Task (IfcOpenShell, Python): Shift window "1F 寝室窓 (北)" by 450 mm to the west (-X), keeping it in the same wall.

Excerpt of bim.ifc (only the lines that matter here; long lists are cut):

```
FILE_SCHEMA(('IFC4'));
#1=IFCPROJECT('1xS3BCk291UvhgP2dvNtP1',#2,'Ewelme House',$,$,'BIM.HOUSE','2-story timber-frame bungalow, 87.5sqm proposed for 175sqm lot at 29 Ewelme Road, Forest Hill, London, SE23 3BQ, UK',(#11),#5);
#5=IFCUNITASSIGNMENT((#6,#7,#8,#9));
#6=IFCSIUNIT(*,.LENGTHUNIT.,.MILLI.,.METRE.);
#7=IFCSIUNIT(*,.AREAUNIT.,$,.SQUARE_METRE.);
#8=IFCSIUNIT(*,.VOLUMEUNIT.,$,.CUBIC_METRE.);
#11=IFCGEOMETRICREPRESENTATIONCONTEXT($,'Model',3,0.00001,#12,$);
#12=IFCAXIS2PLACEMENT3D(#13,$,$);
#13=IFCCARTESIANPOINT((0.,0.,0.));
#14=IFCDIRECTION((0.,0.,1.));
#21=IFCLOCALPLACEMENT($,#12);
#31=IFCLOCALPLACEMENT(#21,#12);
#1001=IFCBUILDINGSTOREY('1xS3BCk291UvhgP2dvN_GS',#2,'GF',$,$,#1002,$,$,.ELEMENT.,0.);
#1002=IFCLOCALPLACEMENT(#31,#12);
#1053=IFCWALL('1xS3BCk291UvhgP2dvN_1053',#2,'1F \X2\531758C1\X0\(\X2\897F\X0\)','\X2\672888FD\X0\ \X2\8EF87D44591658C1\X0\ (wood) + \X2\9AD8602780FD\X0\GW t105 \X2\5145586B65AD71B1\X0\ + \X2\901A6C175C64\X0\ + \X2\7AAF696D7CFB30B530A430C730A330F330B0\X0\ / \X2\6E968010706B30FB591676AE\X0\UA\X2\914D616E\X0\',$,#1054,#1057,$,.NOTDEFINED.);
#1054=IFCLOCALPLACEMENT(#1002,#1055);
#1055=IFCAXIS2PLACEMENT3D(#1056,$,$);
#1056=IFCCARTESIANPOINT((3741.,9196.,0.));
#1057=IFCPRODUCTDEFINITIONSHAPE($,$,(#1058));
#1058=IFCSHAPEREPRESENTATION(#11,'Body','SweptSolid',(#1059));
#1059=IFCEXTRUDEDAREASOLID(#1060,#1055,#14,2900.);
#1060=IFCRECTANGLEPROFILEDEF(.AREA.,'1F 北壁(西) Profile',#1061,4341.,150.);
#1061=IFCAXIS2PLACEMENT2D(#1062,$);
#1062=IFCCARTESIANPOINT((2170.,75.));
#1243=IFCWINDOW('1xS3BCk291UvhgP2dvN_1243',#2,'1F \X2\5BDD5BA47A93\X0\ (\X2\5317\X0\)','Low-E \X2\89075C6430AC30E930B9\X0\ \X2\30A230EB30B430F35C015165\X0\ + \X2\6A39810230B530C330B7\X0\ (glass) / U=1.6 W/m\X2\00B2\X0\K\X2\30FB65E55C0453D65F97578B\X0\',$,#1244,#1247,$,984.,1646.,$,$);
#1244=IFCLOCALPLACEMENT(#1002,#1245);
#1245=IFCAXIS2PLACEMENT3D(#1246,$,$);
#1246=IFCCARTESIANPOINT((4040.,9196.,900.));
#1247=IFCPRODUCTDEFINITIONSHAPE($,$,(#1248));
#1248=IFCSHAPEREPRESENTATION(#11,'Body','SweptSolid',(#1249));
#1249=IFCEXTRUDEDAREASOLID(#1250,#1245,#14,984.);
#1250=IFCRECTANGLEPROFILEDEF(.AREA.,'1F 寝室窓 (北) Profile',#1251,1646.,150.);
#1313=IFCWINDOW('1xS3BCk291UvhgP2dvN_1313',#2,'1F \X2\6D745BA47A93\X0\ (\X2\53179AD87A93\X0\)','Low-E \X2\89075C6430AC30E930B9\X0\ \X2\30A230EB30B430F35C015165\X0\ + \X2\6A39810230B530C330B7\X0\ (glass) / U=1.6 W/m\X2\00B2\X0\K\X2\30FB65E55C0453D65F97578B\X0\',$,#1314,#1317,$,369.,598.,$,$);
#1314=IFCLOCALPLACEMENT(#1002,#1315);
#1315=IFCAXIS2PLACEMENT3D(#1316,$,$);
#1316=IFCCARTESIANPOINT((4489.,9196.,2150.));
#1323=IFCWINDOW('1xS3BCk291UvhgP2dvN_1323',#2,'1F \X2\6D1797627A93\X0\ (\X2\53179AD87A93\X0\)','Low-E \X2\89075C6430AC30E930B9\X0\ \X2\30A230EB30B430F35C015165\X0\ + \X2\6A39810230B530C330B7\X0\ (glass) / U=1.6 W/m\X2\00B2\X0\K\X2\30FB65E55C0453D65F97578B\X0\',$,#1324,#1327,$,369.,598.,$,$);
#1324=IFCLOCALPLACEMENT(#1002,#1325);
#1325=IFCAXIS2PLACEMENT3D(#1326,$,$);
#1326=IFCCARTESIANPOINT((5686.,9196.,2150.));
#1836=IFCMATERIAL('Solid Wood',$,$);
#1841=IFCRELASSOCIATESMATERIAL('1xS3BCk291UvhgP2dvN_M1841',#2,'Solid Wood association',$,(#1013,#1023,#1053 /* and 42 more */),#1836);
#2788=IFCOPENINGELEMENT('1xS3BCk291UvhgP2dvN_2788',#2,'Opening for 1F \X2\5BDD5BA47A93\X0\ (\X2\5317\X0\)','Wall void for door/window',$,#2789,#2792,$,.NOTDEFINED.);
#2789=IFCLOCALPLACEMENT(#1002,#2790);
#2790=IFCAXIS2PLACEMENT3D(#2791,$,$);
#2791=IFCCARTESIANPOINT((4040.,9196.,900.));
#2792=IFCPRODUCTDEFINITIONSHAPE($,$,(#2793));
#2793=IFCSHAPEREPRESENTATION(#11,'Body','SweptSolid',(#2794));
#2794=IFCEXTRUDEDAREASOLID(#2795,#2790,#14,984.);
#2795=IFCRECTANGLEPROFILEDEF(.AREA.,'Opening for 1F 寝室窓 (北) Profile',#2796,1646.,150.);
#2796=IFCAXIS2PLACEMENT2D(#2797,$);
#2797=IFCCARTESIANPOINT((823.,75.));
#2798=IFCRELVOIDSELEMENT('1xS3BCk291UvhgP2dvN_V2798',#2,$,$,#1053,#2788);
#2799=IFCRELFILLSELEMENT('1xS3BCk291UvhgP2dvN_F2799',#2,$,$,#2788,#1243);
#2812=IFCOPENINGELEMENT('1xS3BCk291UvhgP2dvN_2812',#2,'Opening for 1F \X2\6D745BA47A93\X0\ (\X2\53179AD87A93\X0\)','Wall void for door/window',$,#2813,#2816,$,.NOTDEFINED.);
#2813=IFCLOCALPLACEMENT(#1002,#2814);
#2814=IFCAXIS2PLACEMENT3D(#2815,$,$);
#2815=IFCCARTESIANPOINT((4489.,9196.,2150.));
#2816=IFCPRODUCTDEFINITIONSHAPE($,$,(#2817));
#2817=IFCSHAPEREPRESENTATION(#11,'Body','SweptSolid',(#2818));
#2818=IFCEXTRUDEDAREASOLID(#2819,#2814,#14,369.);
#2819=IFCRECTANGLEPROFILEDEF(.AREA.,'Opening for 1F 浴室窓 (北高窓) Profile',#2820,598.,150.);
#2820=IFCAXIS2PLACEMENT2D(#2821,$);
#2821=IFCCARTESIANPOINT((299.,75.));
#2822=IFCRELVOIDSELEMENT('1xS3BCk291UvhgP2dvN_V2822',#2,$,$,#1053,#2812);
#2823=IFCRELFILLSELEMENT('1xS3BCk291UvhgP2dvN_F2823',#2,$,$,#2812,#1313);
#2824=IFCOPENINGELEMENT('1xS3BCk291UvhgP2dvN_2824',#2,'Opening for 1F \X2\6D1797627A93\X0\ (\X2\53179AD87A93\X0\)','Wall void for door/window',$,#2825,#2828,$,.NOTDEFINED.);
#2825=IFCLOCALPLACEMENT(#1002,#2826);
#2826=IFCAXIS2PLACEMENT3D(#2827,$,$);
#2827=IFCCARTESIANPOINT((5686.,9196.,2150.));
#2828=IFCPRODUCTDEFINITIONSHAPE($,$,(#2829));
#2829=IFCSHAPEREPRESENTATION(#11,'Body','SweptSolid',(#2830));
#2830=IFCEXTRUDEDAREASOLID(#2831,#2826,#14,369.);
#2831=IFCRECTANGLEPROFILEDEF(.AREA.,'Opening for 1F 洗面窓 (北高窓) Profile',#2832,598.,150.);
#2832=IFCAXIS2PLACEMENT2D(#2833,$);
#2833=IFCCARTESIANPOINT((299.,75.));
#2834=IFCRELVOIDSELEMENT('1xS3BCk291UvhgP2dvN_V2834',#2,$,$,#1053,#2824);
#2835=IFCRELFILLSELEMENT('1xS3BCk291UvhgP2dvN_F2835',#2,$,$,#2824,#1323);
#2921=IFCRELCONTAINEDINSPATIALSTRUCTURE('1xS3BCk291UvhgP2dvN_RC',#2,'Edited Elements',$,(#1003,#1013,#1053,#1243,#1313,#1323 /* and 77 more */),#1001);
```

```python
import ifcopenshell
import ifcopenshell.api.geometry
import ifcopenshell.util.placement
import ifcopenshell.util.unit

model = ifcopenshell.open("bim.ifc")
unit_scale = ifcopenshell.util.unit.calculate_unit_scale(model)

window = model.by_guid("1xS3BCk291UvhgP2dvN_1243")
opening = window.FillsVoids[0].RelatingOpeningElement
wall = opening.VoidsElements[0].RelatingBuildingElement

wall_matrix = ifcopenshell.util.placement.get_local_placement(wall.ObjectPlacement)
shift = wall_matrix[:3, 0] * -0.45 / unit_scale
before = ifcopenshell.util.placement.get_local_placement(window.ObjectPlacement)[:3, 3].copy()

# The window is not placed relative to its opening, so move both.
for product in (opening, window):
    matrix = ifcopenshell.util.placement.get_local_placement(product.ObjectPlacement)
    matrix[:3, 3] += shift
    ifcopenshell.api.geometry.edit_object_placement(model, product=product, matrix=matrix, is_si=False)

after = ifcopenshell.util.placement.get_local_placement(window.ObjectPlacement)[:3, 3]
print("window moved by", (after - before).round(3) + 0.0)

model.write("bim_updated.ifc")
```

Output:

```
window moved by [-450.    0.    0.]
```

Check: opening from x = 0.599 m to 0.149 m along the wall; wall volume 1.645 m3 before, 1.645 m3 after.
